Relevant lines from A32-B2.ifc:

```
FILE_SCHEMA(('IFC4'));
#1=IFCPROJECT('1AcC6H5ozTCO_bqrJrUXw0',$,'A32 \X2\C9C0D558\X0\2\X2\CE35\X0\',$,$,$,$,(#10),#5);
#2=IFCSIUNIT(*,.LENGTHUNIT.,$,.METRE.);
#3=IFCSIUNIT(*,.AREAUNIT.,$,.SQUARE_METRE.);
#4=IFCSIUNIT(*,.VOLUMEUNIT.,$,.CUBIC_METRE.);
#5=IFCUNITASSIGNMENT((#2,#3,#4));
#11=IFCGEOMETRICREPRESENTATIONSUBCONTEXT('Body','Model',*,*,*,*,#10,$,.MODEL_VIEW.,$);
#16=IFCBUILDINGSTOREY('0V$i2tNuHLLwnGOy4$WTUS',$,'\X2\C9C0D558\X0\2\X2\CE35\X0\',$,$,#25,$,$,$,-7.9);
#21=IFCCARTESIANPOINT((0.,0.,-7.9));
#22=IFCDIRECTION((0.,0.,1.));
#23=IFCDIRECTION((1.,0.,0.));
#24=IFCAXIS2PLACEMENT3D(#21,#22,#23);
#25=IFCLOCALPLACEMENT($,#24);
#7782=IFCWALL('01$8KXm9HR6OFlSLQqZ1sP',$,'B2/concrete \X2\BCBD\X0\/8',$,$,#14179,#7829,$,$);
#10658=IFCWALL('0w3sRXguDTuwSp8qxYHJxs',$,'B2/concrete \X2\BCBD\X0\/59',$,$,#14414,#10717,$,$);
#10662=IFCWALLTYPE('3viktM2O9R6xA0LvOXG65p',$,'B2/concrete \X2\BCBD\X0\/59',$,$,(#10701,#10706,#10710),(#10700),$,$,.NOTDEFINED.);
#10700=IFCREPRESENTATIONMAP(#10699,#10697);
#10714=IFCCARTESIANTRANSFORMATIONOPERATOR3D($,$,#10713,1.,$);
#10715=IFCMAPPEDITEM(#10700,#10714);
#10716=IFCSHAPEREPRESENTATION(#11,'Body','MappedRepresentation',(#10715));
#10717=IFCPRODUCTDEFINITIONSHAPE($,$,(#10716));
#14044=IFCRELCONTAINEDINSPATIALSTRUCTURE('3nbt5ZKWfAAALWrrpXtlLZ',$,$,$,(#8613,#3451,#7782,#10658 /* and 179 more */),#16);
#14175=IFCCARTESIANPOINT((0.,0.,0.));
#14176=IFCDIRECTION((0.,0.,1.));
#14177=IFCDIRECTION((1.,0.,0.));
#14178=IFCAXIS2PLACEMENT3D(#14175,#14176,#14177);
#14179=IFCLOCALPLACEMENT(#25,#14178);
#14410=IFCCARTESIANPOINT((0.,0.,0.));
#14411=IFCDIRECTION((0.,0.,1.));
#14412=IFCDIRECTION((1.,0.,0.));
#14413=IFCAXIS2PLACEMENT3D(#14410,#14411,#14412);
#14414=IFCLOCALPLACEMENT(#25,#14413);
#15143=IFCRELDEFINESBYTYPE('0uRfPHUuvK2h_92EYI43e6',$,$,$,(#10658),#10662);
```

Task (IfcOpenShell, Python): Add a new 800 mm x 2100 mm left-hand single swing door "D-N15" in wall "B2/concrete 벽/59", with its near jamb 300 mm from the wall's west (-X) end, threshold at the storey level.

```python
import numpy as np
import ifcopenshell
import ifcopenshell.api.feature
import ifcopenshell.api.geometry
import ifcopenshell.api.root
import ifcopenshell.api.spatial
import ifcopenshell.geom
import ifcopenshell.util.element
import ifcopenshell.util.placement
import ifcopenshell.util.representation
import ifcopenshell.util.shape
import ifcopenshell.util.unit

model = ifcopenshell.open("A32-B2.ifc")
unit_scale = ifcopenshell.util.unit.calculate_unit_scale(model)
settings = ifcopenshell.geom.settings()


def volume(element):
    """Net volume in cubic metres, openings subtracted."""
    shape = ifcopenshell.geom.create_shape(settings, element)
    return ifcopenshell.util.shape.get_volume(shape.geometry)


wall = model.by_guid("0w3sRXguDTuwSp8qxYHJxs")
storey = ifcopenshell.util.element.get_container(wall, ifc_class="IfcBuildingStorey")
context = ifcopenshell.util.representation.get_context(model, "Model", "Body", "MODEL_VIEW")
before = volume(wall)

width, height, from_end, sill = 0.8, 2.1, 0.3, 0.0  # metres

# The wall runs along its own X axis, and the end named is its -X end.
wall_shape = ifcopenshell.geom.create_shape(settings, wall)
x, y, z = ifcopenshell.util.shape.get_vertices(wall_shape.geometry).T
start = x.min() + from_end
face, thickness = float(y.min()), float(y.max() - y.min())
wall_matrix = ifcopenshell.util.placement.get_local_placement(wall.ObjectPlacement)
level = ifcopenshell.util.placement.get_local_placement(storey.ObjectPlacement)[2, 3]


def in_wall(x, y):
    """Placement at x, y metres in the wall's axes, at sill height."""
    matrix = wall_matrix.copy()
    matrix[:, 3] = wall_matrix @ np.array([x / unit_scale, y / unit_scale, 0.0, 1.0])
    matrix[2, 3] = level + sill / unit_scale
    return matrix


# Opening: a box that overshoots both wall faces by 50 mm.
opening = ifcopenshell.api.root.create_entity(model, ifc_class="IfcOpeningElement", predefined_type="OPENING")
box = ifcopenshell.api.geometry.add_wall_representation(
    model, context=context, length=width, height=height, thickness=thickness + 0.1
)
ifcopenshell.api.geometry.assign_representation(model, product=opening, representation=box)
ifcopenshell.api.geometry.edit_object_placement(model, product=opening, matrix=in_wall(start, face - 0.05), is_si=False)
ifcopenshell.api.feature.add_feature(model, feature=opening, element=wall)

door = ifcopenshell.api.root.create_entity(model, ifc_class="IfcDoor", name="D-N15", predefined_type="DOOR")
door.OverallWidth, door.OverallHeight = width / unit_scale, height / unit_scale
door.OperationType = "SINGLE_SWING_LEFT"
body = ifcopenshell.api.geometry.add_door_representation(
    model,
    context=context,
    overall_width=door.OverallWidth,
    overall_height=door.OverallHeight,
    operation_type="SINGLE_SWING_LEFT",
    lining_properties={"LiningDepth": thickness / unit_scale, "ThresholdDepth": thickness / unit_scale},
)
ifcopenshell.api.geometry.assign_representation(model, product=door, representation=body)
ifcopenshell.api.spatial.assign_container(model, products=[door], relating_structure=storey)
ifcopenshell.api.feature.add_filling(model, opening=opening, element=door)

# The lining spans the wall, so the door starts at the wall face.
ifcopenshell.api.geometry.edit_object_placement(model, product=door, matrix=in_wall(start, face), is_si=False)

after = volume(wall)

print(f"wall volume {before:.3f} -> {after:.3f} m3")

model.write("A32-B2_rev.ifc")
```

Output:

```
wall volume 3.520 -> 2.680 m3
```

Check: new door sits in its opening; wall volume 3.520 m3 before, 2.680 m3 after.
